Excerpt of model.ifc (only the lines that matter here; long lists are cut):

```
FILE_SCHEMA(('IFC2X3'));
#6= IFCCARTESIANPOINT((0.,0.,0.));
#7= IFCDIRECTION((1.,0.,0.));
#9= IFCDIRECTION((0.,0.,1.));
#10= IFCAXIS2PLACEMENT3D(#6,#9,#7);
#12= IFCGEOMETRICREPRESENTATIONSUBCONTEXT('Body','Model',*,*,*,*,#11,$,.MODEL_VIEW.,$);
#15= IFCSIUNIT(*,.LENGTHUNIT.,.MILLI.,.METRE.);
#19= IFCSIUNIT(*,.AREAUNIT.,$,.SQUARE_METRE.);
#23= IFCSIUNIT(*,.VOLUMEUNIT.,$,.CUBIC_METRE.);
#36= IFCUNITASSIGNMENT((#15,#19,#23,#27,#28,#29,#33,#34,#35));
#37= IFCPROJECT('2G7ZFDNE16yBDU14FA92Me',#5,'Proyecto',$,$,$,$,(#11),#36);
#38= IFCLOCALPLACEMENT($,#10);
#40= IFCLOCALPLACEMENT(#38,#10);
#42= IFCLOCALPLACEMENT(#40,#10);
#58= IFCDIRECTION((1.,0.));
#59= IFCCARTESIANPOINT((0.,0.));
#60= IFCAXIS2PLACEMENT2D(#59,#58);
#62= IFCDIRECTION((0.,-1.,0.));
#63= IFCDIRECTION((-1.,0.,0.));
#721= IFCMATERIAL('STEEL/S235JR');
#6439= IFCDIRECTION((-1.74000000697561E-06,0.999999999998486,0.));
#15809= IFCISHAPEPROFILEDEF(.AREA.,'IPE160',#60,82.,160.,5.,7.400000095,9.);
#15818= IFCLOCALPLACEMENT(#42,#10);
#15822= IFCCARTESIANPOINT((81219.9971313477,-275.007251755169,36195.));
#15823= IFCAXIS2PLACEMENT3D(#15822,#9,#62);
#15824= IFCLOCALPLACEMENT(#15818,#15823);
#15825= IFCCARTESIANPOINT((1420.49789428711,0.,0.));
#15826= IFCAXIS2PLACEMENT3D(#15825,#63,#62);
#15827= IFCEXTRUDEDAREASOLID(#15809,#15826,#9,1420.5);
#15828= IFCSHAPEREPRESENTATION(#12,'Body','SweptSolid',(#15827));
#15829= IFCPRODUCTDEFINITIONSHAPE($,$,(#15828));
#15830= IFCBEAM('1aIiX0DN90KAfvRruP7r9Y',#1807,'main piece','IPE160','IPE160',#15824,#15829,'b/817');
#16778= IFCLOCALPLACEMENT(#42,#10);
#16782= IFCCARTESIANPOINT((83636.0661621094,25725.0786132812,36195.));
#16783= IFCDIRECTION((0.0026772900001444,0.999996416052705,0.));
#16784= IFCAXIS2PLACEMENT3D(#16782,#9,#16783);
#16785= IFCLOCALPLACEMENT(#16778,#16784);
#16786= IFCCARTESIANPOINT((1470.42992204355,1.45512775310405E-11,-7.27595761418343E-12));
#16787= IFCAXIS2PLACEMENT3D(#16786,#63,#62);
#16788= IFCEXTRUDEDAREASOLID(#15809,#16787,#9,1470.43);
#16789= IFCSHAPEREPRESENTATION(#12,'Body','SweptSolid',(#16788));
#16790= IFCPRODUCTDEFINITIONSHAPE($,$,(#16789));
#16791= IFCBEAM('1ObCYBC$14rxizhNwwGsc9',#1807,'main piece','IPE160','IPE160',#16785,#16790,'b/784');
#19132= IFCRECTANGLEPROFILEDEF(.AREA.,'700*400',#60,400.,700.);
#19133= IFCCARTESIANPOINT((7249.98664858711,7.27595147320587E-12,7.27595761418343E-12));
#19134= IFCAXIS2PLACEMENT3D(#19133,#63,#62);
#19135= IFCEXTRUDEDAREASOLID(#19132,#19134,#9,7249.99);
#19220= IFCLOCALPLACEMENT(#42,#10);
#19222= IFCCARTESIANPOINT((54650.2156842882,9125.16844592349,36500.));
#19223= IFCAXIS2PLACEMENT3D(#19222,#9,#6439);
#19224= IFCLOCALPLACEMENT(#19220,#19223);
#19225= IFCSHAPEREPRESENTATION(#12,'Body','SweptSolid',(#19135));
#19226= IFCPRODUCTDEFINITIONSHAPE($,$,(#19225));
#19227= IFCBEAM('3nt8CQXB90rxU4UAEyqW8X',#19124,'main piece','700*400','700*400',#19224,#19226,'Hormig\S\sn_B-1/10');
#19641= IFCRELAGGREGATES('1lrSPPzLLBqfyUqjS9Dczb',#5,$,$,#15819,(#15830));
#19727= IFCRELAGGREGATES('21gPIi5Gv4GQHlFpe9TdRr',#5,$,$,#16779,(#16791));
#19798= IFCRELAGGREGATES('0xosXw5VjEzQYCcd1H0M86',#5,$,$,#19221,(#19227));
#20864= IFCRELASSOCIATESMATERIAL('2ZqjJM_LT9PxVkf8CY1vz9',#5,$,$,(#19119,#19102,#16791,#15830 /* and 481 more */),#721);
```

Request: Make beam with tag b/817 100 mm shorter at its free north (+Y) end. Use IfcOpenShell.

```python
import ifcopenshell
import ifcopenshell.util.representation
import ifcopenshell.util.unit

model = ifcopenshell.open("model.ifc")
unit_scale = ifcopenshell.util.unit.calculate_unit_scale(model)

member = model.by_guid("1aIiX0DN90KAfvRruP7r9Y")
change = -0.1 / unit_scale

# The extrusion runs towards the end named, so only its depth changes.
body = ifcopenshell.util.representation.get_representation(member, "Model", "Body")
solid = body.Items[0]
old_length = solid.Depth
solid.Depth += change

print(f"length {old_length:g} -> {solid.Depth:g}")

model.write("model_v2.ifc")
```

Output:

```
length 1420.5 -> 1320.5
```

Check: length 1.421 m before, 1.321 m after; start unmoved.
